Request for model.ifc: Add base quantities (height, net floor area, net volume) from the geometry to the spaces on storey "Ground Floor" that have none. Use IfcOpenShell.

First a look at what the model holds.

```python
import ifcopenshell
import ifcopenshell.util.element
import ifcopenshell.util.unit

model = ifcopenshell.open("model.ifc")
print(model.schema)
for unit_type in ("LENGTHUNIT", "AREAUNIT", "VOLUMEUNIT"):
    print(unit_type, ifcopenshell.util.unit.calculate_unit_scale(model, unit_type))
storey = next(s for s in model.by_type("IfcBuildingStorey") if s.Name == "Ground Floor")
spaces = [e for e in ifcopenshell.util.element.get_decomposition(storey) if e.is_a("IfcSpace")]
for e in sorted(spaces, key=lambda e: e.id()):
    print(e.id(), e.is_a(), e.Name, list(ifcopenshell.util.element.get_psets(e, qtos_only=True)), sep=" | ")
```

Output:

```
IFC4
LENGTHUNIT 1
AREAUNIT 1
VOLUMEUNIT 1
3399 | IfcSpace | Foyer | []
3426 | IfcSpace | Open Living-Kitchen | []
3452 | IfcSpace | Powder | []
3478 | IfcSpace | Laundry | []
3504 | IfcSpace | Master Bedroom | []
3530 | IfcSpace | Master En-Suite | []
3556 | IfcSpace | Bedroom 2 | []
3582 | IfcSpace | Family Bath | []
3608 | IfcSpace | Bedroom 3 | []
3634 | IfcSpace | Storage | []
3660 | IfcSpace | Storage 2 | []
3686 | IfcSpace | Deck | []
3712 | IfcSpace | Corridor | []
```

```python
import ifcopenshell
import ifcopenshell.api.pset
import ifcopenshell.geom
import ifcopenshell.util.element
import ifcopenshell.util.shape
import ifcopenshell.util.unit

model = ifcopenshell.open("model.ifc")
unit_scale = ifcopenshell.util.unit.calculate_unit_scale(model)
area_scale = ifcopenshell.util.unit.calculate_unit_scale(model, "AREAUNIT")
volume_scale = ifcopenshell.util.unit.calculate_unit_scale(model, "VOLUMEUNIT")
settings = ifcopenshell.geom.settings()

storey = next(s for s in model.by_type("IfcBuildingStorey") if s.Name == "Ground Floor")
spaces = [e for e in ifcopenshell.util.element.get_decomposition(storey) if e.is_a("IfcSpace")]

for e in sorted(spaces, key=lambda e: e.id()):
    if ifcopenshell.util.element.get_psets(e, qtos_only=True, should_inherit=False):
        continue
    # Geometry comes back in metres, in the element's own axes.
    shape = ifcopenshell.geom.create_shape(settings, e)
    values = {
        "Height": ifcopenshell.util.shape.get_z(shape.geometry) / unit_scale,
        "NetFloorArea": ifcopenshell.util.shape.get_footprint_area(shape.geometry) / area_scale,
        "NetVolume": ifcopenshell.util.shape.get_volume(shape.geometry) / volume_scale,
    }
    qto = ifcopenshell.api.pset.add_qto(model, product=e, name="Qto_SpaceBaseQuantities")
    ifcopenshell.api.pset.edit_qto(model, qto=qto, properties=values)
    print(e.id(), {k: round(v, 3) for k, v in values.items()})

model.write("model_updated.ifc")
```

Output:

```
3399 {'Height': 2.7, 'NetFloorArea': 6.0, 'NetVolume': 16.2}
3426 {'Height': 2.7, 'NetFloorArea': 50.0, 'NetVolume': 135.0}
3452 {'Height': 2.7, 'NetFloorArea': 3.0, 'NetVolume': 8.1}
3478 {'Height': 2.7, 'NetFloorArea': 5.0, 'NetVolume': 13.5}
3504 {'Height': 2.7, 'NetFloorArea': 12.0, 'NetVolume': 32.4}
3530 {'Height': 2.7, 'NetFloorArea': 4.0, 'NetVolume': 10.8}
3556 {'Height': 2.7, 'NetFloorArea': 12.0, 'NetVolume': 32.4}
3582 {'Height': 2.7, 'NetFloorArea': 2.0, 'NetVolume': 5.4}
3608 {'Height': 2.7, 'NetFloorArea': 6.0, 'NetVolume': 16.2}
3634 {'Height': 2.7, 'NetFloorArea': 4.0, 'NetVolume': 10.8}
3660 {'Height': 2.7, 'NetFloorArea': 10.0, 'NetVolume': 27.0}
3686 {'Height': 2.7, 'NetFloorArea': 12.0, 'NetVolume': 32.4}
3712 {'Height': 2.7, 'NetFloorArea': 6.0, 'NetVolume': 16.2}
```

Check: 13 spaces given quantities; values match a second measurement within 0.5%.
